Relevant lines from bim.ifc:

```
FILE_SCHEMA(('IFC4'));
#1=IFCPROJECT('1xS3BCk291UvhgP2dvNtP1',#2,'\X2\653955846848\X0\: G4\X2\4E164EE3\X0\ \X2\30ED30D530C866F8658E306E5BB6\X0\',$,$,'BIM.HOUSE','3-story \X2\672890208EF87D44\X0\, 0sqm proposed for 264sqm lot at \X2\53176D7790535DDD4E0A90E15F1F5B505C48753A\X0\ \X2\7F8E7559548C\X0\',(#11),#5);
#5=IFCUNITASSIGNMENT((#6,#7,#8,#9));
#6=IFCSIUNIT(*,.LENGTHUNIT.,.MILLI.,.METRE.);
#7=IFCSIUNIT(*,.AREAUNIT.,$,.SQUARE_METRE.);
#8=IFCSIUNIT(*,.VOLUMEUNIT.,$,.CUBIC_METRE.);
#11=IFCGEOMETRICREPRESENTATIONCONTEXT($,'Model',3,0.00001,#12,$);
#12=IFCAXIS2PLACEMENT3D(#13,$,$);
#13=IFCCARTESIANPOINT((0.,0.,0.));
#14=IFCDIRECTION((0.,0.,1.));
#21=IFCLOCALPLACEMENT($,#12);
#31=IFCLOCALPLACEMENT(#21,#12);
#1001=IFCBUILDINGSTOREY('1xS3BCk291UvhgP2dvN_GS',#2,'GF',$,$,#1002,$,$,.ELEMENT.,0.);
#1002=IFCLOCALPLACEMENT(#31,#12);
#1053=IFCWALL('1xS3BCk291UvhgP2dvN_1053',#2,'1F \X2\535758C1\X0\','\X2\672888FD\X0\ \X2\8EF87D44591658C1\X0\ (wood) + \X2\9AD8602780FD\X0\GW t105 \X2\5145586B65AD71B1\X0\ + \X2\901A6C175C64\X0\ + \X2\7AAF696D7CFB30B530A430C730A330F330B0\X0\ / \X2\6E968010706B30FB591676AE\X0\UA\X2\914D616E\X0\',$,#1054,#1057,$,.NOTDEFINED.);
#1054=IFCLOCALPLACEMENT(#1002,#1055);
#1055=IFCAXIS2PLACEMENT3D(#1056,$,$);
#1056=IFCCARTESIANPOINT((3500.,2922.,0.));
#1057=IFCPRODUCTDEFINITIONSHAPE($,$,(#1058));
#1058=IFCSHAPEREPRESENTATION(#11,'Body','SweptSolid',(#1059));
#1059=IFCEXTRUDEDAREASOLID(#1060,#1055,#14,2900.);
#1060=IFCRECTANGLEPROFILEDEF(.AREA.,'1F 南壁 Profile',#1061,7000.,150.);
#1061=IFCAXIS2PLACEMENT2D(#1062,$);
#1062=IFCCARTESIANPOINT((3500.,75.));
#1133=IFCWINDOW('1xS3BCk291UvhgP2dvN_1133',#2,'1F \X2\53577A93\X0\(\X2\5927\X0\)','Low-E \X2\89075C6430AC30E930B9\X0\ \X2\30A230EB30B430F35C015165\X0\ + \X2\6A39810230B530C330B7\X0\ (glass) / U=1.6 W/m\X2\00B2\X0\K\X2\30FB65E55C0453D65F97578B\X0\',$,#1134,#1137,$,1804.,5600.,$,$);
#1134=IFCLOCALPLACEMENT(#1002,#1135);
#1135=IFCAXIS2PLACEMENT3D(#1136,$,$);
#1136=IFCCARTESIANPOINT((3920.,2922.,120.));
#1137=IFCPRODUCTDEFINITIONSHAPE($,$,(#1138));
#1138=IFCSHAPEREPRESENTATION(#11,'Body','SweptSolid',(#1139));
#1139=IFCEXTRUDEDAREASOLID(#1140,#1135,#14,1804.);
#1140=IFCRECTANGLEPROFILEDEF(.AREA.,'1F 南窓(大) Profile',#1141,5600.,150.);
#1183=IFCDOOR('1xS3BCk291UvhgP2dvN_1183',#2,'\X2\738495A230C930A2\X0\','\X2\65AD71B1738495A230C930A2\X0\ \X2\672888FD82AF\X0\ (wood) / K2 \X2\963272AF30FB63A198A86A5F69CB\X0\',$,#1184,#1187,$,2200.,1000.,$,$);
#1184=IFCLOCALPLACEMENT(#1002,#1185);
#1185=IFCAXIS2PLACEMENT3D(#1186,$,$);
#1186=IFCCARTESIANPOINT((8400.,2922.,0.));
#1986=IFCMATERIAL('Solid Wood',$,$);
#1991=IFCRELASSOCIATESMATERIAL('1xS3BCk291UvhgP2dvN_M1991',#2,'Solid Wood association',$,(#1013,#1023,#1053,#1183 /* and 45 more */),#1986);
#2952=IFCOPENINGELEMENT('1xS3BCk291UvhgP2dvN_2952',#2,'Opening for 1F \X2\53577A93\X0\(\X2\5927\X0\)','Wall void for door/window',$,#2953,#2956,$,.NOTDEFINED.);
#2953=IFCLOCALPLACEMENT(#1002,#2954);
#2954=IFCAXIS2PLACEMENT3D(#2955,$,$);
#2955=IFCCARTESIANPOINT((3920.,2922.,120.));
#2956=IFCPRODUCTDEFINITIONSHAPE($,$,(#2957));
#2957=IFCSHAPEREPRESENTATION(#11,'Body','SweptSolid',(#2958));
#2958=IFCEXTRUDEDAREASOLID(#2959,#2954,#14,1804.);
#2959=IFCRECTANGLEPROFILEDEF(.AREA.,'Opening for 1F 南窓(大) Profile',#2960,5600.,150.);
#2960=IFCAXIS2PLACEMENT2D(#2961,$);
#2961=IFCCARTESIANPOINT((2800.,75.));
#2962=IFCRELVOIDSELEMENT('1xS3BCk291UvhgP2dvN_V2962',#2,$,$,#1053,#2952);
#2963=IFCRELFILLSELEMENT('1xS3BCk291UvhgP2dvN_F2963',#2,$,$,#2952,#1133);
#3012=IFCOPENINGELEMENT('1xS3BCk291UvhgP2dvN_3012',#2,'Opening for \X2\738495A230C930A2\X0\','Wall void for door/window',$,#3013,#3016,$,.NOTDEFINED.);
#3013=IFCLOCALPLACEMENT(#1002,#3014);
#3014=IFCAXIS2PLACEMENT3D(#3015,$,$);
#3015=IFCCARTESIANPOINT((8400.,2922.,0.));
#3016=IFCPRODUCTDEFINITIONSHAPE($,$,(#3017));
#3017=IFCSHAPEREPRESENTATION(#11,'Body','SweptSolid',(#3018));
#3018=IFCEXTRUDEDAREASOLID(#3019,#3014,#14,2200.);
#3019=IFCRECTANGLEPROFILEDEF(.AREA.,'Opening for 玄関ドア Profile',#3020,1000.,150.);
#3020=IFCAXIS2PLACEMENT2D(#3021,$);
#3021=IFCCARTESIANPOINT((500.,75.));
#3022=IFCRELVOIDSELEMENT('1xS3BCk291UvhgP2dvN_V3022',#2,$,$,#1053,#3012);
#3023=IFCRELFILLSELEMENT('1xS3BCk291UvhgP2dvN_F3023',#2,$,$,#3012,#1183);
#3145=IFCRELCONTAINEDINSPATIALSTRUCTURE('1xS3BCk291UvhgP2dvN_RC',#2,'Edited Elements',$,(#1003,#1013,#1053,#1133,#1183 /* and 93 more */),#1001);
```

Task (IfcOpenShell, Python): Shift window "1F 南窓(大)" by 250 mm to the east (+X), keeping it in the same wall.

```python
import ifcopenshell
import ifcopenshell.api.geometry
import ifcopenshell.util.placement

model = ifcopenshell.open("bim.ifc")

window = model.by_guid("1xS3BCk291UvhgP2dvN_1133")
opening = window.FillsVoids[0].RelatingOpeningElement
wall = opening.VoidsElements[0].RelatingBuildingElement

wall_matrix = ifcopenshell.util.placement.get_local_placement(wall.ObjectPlacement)
shift = wall_matrix[:3, 0] * 250.0
before = ifcopenshell.util.placement.get_local_placement(window.ObjectPlacement)[:3, 3].copy()

# The window is not placed relative to its opening, so move both.
for product in (opening, window):
    matrix = ifcopenshell.util.placement.get_local_placement(product.ObjectPlacement)
    matrix[:3, 3] += shift
    ifcopenshell.api.geometry.edit_object_placement(model, product=product, matrix=matrix, is_si=False)

after = ifcopenshell.util.placement.get_local_placement(window.ObjectPlacement)[:3, 3]
print("window moved by", (after - before).round(3) + 0.0)

model.write("bim_edited.ifc")
```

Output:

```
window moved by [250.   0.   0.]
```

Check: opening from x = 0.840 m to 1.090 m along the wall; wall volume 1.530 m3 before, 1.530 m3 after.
